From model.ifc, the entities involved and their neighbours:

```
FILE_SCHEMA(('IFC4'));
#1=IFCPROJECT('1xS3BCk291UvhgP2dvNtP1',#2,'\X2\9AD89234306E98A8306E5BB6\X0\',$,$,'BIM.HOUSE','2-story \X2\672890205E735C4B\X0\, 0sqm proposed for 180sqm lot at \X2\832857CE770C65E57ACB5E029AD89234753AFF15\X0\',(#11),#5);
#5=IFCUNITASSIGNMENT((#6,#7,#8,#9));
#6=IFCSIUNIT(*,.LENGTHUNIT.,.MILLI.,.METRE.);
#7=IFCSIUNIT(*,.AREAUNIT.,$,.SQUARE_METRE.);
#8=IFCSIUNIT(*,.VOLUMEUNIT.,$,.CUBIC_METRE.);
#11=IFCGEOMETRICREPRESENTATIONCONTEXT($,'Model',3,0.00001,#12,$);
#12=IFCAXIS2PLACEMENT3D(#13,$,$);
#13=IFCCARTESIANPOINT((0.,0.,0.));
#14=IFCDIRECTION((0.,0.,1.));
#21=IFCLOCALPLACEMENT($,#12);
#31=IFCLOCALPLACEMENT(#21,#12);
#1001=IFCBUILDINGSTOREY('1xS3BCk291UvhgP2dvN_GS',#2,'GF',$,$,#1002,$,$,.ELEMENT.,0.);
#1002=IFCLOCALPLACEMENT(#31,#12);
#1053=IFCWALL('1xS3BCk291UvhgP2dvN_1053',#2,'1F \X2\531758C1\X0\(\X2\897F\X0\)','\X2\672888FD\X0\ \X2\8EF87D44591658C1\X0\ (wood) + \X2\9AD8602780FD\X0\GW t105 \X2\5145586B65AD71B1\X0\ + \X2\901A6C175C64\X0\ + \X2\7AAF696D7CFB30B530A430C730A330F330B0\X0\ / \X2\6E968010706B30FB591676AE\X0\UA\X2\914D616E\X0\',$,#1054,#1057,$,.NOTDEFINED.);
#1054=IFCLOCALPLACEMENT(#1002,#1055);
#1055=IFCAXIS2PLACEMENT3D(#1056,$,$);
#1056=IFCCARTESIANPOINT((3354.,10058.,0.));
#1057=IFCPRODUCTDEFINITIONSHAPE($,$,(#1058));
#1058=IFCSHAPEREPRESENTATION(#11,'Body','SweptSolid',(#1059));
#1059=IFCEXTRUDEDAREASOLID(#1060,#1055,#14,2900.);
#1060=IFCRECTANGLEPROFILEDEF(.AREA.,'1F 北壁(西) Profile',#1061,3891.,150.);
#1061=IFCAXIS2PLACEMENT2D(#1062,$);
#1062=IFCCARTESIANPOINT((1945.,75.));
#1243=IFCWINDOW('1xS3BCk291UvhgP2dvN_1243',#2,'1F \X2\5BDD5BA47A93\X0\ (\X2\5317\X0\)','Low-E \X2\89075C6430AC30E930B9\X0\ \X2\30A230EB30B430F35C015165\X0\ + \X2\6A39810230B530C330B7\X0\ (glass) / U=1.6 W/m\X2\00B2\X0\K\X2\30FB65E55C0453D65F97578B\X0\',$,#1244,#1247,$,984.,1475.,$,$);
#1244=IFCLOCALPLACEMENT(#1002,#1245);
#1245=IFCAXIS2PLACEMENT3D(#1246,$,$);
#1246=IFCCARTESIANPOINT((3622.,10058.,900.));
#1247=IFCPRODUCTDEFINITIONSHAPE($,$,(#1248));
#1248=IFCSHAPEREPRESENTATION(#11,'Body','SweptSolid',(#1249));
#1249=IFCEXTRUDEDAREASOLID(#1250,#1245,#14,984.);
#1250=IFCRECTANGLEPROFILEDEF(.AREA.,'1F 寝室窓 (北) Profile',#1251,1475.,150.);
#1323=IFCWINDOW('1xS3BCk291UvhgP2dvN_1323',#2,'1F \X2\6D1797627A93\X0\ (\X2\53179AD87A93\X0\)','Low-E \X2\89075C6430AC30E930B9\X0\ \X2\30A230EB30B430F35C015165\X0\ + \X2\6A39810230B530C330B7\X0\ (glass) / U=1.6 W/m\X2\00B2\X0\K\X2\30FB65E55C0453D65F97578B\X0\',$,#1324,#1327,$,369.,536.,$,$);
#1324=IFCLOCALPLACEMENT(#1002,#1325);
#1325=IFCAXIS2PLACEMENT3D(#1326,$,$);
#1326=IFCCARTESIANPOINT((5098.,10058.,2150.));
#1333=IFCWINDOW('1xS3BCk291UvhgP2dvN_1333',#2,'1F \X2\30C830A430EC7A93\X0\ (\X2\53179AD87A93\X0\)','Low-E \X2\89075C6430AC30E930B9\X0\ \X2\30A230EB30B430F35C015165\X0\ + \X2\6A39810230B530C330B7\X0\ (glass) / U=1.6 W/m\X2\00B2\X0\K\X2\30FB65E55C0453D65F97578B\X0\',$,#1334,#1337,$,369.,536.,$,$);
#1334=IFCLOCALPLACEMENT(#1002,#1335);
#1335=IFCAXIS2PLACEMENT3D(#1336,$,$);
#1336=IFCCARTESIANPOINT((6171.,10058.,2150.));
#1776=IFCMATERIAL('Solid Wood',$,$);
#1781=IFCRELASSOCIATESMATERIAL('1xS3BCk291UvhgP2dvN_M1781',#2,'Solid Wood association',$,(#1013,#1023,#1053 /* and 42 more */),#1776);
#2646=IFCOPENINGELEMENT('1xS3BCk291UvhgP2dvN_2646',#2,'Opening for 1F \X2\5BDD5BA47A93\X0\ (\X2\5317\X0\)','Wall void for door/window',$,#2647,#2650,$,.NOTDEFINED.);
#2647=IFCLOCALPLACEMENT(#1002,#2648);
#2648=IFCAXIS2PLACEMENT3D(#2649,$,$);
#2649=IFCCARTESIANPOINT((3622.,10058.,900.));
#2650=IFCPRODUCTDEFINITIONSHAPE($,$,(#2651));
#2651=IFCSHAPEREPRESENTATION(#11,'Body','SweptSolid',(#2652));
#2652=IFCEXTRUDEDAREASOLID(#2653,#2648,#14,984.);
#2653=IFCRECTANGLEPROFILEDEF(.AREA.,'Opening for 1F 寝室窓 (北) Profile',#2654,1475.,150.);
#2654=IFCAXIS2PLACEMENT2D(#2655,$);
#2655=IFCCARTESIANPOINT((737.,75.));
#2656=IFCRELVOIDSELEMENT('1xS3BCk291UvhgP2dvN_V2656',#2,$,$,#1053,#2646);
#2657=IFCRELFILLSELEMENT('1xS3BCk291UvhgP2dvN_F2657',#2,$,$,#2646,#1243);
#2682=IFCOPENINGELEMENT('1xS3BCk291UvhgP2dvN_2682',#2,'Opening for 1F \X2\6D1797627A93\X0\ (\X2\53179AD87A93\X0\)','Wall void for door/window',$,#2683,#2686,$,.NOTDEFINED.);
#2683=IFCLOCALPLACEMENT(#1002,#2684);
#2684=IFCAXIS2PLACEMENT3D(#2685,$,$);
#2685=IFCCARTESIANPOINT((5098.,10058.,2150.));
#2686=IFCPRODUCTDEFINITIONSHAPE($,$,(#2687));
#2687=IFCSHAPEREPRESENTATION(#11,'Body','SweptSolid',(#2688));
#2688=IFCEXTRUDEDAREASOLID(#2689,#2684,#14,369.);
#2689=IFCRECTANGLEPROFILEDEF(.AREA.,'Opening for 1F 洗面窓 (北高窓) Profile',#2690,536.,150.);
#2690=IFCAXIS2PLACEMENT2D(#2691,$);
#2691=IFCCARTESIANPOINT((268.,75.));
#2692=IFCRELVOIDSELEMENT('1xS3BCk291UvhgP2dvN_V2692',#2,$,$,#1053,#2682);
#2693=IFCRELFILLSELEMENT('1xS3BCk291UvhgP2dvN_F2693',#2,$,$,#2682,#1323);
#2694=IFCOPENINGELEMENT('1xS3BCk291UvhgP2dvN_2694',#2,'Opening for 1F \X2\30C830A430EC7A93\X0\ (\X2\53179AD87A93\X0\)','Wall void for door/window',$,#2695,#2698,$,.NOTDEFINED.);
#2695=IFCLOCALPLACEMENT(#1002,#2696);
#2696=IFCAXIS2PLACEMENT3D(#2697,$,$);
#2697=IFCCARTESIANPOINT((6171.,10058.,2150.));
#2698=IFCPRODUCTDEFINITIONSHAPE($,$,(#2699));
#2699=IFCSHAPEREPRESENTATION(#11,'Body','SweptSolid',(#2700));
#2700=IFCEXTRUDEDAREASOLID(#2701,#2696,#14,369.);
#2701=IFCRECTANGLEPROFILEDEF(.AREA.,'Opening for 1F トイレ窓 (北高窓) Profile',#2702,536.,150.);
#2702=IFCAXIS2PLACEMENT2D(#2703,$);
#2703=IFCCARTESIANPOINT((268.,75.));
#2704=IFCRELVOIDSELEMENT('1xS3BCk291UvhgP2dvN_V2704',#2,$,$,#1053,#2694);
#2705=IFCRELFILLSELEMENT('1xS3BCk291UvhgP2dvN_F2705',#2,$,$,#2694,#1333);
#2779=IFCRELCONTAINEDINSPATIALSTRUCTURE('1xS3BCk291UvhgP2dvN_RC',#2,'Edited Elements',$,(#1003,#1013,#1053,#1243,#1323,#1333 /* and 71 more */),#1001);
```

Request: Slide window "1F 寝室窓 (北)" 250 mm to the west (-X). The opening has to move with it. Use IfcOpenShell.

```python
import ifcopenshell
import ifcopenshell.api.geometry
import ifcopenshell.util.placement
import ifcopenshell.util.unit

model = ifcopenshell.open("model.ifc")
unit_scale = ifcopenshell.util.unit.calculate_unit_scale(model)

window = model.by_guid("1xS3BCk291UvhgP2dvN_1243")
opening = window.FillsVoids[0].RelatingOpeningElement
wall = opening.VoidsElements[0].RelatingBuildingElement

wall_matrix = ifcopenshell.util.placement.get_local_placement(wall.ObjectPlacement)
shift = wall_matrix[:3, 0] * -0.25 / unit_scale
before = ifcopenshell.util.placement.get_local_placement(window.ObjectPlacement)[:3, 3].copy()

# The window is not placed relative to its opening, so move both.
for product in (opening, window):
    matrix = ifcopenshell.util.placement.get_local_placement(product.ObjectPlacement)
    matrix[:3, 3] += shift
    ifcopenshell.api.geometry.edit_object_placement(model, product=product, matrix=matrix, is_si=False)

after = ifcopenshell.util.placement.get_local_placement(window.ObjectPlacement)[:3, 3]
print("window moved by", (after - before).round(3) + 0.0)

model.write("model_updated.ifc")
```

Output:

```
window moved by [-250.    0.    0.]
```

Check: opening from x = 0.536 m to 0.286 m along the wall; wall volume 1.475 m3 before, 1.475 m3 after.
